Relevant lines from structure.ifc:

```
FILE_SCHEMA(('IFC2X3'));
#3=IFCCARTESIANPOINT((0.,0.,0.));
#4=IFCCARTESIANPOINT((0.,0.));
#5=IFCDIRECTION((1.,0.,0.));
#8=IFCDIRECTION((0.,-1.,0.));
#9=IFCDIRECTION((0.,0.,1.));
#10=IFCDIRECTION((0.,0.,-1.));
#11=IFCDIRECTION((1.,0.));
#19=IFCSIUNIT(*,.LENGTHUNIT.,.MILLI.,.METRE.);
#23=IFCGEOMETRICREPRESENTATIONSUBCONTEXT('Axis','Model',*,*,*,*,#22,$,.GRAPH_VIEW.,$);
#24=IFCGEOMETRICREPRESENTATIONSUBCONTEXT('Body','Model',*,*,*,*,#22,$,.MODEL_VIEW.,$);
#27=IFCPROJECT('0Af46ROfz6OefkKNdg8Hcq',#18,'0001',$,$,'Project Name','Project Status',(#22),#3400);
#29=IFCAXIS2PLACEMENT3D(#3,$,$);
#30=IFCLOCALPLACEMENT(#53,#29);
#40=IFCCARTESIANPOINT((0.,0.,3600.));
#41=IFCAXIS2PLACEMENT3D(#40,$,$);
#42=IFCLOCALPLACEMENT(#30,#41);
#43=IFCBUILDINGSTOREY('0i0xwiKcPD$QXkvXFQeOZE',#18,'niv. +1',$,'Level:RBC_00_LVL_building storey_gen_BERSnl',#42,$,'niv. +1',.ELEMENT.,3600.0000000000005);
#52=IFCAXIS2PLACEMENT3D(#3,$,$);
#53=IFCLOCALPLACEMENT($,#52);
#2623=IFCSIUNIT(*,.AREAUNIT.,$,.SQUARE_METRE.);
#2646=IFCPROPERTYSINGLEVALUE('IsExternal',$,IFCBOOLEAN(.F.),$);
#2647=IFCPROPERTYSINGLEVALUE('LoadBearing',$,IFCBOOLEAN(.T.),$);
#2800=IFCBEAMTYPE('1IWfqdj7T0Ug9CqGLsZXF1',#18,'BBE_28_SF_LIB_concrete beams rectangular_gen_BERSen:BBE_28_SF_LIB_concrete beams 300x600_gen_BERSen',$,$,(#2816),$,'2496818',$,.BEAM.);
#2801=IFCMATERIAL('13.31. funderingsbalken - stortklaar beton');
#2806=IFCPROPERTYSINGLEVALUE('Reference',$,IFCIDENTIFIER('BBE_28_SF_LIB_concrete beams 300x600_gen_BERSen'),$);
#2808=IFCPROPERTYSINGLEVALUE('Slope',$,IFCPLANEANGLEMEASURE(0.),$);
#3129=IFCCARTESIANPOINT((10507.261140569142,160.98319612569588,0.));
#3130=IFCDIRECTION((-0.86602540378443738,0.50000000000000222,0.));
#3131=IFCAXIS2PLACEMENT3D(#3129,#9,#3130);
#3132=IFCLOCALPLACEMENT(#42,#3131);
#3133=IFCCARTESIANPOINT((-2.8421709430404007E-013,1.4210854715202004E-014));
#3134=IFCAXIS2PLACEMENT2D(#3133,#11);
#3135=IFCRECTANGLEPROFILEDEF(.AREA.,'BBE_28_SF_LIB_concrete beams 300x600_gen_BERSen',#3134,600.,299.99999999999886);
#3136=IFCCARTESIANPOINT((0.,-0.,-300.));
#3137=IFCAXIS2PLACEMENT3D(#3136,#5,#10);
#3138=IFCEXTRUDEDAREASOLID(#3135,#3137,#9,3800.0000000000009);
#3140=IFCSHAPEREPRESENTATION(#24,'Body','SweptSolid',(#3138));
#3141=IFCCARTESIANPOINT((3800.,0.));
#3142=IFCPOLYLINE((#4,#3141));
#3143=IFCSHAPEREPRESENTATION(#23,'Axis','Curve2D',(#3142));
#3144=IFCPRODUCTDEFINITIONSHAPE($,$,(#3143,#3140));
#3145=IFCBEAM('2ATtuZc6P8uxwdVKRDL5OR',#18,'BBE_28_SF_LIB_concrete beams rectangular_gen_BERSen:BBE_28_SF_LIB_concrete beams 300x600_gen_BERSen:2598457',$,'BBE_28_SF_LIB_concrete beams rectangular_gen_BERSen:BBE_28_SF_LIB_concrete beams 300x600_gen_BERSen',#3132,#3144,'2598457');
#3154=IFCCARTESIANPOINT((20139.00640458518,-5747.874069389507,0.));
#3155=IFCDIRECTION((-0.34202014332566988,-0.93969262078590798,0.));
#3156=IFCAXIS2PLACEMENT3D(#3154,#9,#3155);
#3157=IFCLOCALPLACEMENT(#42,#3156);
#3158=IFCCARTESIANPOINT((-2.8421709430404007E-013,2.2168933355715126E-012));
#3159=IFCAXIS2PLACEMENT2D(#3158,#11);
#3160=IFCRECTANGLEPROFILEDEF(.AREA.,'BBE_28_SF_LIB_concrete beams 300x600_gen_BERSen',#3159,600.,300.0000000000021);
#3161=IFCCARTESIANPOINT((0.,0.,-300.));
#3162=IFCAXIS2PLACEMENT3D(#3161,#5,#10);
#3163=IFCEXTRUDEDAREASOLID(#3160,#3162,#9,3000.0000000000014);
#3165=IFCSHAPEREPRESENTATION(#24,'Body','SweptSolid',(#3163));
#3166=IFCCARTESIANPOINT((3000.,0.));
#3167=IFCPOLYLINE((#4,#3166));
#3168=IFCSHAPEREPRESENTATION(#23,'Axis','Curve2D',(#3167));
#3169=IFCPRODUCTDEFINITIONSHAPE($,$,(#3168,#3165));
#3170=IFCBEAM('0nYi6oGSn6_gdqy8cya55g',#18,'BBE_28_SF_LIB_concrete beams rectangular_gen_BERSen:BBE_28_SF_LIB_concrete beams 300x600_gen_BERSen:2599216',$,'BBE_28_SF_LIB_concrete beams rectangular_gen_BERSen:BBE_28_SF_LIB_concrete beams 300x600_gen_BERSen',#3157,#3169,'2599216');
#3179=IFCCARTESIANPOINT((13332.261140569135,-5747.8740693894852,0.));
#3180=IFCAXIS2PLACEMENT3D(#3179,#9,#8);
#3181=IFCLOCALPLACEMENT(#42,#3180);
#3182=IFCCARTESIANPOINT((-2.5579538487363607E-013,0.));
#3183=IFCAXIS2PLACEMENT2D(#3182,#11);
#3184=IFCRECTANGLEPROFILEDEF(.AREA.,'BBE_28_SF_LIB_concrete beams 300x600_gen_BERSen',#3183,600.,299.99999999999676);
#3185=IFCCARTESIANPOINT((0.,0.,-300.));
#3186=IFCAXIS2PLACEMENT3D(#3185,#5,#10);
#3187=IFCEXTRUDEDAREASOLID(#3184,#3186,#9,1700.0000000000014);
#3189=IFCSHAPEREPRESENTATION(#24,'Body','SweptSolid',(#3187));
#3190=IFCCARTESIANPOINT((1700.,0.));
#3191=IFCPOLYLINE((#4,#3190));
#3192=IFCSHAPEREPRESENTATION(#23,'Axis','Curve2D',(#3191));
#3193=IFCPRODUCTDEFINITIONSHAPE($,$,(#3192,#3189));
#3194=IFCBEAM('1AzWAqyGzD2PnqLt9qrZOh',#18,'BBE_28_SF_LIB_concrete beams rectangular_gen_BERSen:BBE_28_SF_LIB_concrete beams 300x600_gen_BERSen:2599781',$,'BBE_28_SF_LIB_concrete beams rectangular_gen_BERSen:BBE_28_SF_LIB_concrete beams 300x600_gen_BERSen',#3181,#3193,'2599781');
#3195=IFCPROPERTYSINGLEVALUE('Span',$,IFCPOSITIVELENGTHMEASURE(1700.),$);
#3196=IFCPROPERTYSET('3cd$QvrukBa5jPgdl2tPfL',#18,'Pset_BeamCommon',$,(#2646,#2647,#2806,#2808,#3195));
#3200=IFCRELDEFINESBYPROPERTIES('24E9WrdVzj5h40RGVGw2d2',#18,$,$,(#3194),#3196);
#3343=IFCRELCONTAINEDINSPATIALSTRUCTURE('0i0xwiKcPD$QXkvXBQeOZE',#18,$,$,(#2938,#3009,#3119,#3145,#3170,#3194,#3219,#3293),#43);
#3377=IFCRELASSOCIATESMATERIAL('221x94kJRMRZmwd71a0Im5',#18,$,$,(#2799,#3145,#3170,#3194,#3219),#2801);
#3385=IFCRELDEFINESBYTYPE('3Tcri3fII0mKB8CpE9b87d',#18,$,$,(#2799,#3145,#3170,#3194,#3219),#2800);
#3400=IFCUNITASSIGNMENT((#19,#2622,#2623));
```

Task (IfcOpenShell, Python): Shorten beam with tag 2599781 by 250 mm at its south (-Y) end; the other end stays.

```python
import numpy as np
import ifcopenshell
import ifcopenshell.api.pset
import ifcopenshell.util.element
import ifcopenshell.util.representation

model = ifcopenshell.open("structure.ifc")

member = model.by_guid("1AzWAqyGzD2PnqLt9qrZOh")
change = -250.0

# The extrusion runs towards the end named, so only its depth changes.
body = ifcopenshell.util.representation.get_representation(member, "Model", "Body")
solid = body.Items[0]
old_length = solid.Depth
solid.Depth += change

# Move the axis end point with it.
axis = next(r for r in member.Representation.Representations if r.RepresentationIdentifier == "Axis").Items[0]
start, end = (np.array(p.Coordinates) for p in axis.Points)
end = end + (end - start) / np.linalg.norm(end - start) * change
point = model.createIfcCartesianPoint(end.tolist())
axis.Points = [axis.Points[0], point]

# Update the stored length and volume.
pset = model.by_id(ifcopenshell.util.element.get_pset(member, "Pset_BeamCommon", should_inherit=False)["id"])
ifcopenshell.api.pset.edit_pset(model, pset=pset, properties={
    "Span": model.create_entity("IfcPositiveLengthMeasure", solid.Depth),
})

print(f"length {old_length:g} -> {solid.Depth:g}")

model.write("structure_v2.ifc")
```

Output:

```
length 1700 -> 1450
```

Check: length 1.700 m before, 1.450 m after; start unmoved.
